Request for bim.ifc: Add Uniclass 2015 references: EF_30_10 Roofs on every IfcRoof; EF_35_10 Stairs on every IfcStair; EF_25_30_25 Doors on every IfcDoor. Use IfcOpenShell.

First a look at what the model holds.

```python
import ifcopenshell

model = ifcopenshell.open("bim.ifc")
print(model.schema)
print("classifications:", [c.Name for c in model.by_type("IfcClassification")])
for ifc_class in ("IfcDoor", "IfcRoof", "IfcStair", "IfcWall", "IfcWindow"):
    print(ifc_class, len(model.by_type(ifc_class)))
```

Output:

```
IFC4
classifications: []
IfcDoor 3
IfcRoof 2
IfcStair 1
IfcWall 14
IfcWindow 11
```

```python
import ifcopenshell
import ifcopenshell.api.classification

model = ifcopenshell.open("bim.ifc")

system = ifcopenshell.api.classification.add_classification(model, classification="Uniclass 2015")

codes = {
    "IfcRoof": ("EF_30_10", "Roofs"),
    "IfcStair": ("EF_35_10", "Stairs"),
    "IfcDoor": ("EF_25_30_25", "Doors"),
}
for ifc_class, (code, name) in codes.items():
    products = model.by_type(ifc_class)
    ifcopenshell.api.classification.add_reference(
        model, products=products, classification=system, identification=code, name=name
    )
    print(code, len(products))

model.write("bim_edited.ifc")
```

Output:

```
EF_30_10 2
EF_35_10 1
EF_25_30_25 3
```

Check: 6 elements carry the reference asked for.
